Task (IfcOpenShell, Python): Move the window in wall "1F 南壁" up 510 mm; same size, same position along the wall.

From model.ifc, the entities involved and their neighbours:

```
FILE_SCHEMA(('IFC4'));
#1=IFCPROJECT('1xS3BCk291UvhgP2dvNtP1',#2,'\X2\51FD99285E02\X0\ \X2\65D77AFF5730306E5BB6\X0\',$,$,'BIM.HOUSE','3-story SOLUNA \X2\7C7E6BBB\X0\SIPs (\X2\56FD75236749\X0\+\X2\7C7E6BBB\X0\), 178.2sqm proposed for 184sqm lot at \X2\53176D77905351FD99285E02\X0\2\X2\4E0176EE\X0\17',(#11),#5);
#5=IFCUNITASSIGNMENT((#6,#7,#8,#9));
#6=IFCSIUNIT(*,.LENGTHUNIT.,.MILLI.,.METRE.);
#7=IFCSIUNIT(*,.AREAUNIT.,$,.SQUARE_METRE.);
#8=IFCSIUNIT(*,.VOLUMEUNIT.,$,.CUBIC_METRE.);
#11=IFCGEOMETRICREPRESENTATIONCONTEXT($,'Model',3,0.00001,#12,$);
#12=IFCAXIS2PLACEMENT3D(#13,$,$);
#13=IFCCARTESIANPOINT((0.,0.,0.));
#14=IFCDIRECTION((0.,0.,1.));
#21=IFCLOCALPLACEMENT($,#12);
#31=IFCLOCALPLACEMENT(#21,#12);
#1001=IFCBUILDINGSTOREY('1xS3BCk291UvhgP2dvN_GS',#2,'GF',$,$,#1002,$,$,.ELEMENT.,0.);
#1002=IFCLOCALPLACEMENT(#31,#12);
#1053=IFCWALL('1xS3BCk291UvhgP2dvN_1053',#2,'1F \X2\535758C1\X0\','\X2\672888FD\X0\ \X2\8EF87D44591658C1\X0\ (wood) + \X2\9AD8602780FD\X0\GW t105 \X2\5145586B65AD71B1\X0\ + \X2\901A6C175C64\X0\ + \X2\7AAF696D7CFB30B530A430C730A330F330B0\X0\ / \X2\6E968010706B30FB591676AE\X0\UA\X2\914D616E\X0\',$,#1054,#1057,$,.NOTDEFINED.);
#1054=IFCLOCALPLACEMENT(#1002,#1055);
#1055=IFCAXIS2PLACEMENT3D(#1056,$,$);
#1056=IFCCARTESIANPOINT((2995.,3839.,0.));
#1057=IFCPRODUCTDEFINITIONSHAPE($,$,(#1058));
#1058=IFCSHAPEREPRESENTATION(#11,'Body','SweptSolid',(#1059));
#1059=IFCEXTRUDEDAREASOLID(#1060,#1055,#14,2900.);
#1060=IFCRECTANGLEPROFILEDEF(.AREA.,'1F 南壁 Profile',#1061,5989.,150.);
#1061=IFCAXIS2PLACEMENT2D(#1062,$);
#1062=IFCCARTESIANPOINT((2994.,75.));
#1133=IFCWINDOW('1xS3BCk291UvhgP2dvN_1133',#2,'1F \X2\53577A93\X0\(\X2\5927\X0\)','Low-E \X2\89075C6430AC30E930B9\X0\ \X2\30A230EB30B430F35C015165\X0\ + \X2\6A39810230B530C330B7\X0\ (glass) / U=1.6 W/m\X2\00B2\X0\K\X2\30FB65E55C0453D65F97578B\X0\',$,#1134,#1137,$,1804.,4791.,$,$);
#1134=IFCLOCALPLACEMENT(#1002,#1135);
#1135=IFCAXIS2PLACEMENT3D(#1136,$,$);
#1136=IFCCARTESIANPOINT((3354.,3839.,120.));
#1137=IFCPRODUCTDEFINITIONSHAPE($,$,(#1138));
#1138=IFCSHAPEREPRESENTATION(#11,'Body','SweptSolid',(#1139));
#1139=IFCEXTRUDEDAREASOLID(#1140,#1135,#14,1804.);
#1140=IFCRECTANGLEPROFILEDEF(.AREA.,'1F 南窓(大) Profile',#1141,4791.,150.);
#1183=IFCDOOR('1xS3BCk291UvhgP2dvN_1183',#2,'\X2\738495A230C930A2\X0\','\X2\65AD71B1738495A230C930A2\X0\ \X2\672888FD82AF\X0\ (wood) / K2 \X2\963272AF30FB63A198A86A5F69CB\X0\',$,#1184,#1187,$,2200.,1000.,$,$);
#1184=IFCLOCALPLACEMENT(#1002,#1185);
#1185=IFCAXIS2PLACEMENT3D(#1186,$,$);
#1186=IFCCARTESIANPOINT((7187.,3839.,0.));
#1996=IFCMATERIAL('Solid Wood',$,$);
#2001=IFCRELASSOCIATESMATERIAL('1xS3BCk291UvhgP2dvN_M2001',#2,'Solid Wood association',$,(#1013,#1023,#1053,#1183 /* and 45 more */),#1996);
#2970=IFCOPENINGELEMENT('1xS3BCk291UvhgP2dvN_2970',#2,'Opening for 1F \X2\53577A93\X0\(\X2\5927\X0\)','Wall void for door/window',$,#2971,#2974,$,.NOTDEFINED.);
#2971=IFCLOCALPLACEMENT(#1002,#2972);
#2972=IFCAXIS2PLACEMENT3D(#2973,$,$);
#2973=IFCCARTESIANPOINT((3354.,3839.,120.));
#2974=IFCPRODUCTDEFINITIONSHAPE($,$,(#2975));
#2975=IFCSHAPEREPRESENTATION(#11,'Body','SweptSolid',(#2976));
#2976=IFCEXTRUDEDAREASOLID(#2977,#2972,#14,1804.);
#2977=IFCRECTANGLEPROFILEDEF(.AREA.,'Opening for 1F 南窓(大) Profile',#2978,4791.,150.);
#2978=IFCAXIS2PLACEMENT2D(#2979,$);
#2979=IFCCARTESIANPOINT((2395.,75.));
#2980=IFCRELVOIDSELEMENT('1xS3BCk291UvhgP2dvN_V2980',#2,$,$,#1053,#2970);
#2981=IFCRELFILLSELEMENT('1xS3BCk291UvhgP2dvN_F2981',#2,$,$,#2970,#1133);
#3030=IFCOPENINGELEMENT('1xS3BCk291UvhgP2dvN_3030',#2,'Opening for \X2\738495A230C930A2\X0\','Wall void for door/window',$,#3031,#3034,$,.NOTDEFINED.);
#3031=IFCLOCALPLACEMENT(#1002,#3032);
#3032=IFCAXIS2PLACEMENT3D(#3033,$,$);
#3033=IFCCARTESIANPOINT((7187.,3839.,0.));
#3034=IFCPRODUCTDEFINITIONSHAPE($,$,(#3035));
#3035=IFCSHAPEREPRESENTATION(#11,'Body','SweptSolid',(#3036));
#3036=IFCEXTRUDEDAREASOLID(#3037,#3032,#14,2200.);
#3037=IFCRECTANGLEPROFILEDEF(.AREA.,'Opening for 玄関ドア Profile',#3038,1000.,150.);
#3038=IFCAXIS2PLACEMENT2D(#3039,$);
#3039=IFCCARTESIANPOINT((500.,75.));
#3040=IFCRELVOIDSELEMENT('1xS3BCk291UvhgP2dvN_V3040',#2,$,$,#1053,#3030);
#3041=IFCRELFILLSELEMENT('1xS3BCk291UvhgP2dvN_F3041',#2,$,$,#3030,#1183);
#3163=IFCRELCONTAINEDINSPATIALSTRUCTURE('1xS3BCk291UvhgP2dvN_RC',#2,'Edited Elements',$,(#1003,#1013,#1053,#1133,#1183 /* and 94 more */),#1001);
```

```python
import numpy as np
import ifcopenshell
import ifcopenshell.api.geometry
import ifcopenshell.util.placement
import ifcopenshell.util.unit

model = ifcopenshell.open("model.ifc")
unit_scale = ifcopenshell.util.unit.calculate_unit_scale(model)

window = model.by_guid("1xS3BCk291UvhgP2dvN_1133")
opening = window.FillsVoids[0].RelatingOpeningElement
dz = 510.0

shift = np.array([0.0, 0.0, dz])
# The window is not placed relative to its opening, so move both.
for product in (opening, window):
    matrix = ifcopenshell.util.placement.get_local_placement(product.ObjectPlacement)
    matrix[:3, 3] += shift
    ifcopenshell.api.geometry.edit_object_placement(model, product=product, matrix=matrix, is_si=False)

print(f"moved by {dz * unit_scale:+.3f} m")

model.write("model-out.ifc")
```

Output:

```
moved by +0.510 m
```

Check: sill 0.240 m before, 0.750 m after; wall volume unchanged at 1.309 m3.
